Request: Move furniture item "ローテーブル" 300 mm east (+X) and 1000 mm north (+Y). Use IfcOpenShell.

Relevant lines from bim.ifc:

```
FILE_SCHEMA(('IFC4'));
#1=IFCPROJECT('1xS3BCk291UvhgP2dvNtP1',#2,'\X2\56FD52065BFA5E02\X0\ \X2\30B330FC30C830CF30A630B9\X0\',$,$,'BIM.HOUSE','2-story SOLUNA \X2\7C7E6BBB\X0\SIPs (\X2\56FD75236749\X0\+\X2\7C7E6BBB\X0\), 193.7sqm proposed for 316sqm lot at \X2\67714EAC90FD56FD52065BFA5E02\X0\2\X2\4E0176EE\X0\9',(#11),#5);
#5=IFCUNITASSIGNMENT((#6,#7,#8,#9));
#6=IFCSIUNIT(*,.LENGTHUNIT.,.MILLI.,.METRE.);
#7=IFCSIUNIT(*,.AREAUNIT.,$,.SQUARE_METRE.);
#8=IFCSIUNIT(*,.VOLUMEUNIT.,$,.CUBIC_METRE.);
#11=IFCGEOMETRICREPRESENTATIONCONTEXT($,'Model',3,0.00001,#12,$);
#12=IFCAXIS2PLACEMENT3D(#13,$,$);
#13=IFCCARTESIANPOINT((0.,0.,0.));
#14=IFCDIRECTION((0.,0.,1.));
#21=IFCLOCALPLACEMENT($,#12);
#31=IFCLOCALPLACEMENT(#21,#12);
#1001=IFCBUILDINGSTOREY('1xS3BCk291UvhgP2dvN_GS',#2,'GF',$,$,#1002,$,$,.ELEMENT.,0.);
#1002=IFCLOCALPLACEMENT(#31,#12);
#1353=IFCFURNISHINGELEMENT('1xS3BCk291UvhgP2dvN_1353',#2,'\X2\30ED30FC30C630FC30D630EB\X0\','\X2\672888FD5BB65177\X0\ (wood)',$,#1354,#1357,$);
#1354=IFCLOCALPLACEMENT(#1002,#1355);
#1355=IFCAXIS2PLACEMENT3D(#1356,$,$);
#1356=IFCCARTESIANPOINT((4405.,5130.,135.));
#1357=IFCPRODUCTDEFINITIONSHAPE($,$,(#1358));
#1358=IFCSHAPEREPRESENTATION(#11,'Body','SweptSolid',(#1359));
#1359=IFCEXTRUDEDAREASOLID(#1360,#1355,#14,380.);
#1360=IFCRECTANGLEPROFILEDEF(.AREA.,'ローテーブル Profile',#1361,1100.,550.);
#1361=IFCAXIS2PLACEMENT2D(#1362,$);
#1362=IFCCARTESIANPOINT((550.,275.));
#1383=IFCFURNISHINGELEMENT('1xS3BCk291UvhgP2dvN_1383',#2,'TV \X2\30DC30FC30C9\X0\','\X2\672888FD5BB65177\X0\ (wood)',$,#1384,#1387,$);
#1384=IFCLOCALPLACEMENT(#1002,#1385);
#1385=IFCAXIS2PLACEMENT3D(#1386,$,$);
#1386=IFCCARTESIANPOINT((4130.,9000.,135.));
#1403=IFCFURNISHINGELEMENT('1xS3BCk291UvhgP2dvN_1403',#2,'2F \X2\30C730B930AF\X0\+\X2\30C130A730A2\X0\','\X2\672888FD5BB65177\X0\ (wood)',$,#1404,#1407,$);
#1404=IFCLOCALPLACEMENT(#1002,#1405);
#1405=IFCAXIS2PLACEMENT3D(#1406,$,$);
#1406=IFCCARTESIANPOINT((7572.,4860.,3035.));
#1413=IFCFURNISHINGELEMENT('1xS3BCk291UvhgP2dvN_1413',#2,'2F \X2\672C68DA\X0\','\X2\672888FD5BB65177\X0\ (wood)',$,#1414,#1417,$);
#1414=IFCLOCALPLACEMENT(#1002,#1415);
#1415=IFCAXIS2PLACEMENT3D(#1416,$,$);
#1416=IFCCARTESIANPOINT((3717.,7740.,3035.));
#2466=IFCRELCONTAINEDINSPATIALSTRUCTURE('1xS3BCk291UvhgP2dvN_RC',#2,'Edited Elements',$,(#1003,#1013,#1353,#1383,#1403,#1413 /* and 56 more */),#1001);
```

```python
import ifcopenshell
import ifcopenshell.api.geometry
import ifcopenshell.util.placement
import ifcopenshell.util.unit

model = ifcopenshell.open("bim.ifc")
unit_scale = ifcopenshell.util.unit.calculate_unit_scale(model)

item = model.by_id(1353)
matrix = ifcopenshell.util.placement.get_local_placement(item.ObjectPlacement)
matrix[0, 3] += 0.3 / unit_scale
matrix[1, 3] += 1 / unit_scale
ifcopenshell.api.geometry.edit_object_placement(model, product=item, matrix=matrix, is_si=False)

print(ifcopenshell.util.placement.get_local_placement(item.ObjectPlacement).round(3) + 0.0)

model.write("bim_updated.ifc")
```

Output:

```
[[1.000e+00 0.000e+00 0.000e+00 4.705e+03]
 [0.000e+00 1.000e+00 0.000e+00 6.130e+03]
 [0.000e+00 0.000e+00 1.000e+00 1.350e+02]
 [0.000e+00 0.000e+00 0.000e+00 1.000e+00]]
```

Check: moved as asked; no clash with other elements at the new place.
